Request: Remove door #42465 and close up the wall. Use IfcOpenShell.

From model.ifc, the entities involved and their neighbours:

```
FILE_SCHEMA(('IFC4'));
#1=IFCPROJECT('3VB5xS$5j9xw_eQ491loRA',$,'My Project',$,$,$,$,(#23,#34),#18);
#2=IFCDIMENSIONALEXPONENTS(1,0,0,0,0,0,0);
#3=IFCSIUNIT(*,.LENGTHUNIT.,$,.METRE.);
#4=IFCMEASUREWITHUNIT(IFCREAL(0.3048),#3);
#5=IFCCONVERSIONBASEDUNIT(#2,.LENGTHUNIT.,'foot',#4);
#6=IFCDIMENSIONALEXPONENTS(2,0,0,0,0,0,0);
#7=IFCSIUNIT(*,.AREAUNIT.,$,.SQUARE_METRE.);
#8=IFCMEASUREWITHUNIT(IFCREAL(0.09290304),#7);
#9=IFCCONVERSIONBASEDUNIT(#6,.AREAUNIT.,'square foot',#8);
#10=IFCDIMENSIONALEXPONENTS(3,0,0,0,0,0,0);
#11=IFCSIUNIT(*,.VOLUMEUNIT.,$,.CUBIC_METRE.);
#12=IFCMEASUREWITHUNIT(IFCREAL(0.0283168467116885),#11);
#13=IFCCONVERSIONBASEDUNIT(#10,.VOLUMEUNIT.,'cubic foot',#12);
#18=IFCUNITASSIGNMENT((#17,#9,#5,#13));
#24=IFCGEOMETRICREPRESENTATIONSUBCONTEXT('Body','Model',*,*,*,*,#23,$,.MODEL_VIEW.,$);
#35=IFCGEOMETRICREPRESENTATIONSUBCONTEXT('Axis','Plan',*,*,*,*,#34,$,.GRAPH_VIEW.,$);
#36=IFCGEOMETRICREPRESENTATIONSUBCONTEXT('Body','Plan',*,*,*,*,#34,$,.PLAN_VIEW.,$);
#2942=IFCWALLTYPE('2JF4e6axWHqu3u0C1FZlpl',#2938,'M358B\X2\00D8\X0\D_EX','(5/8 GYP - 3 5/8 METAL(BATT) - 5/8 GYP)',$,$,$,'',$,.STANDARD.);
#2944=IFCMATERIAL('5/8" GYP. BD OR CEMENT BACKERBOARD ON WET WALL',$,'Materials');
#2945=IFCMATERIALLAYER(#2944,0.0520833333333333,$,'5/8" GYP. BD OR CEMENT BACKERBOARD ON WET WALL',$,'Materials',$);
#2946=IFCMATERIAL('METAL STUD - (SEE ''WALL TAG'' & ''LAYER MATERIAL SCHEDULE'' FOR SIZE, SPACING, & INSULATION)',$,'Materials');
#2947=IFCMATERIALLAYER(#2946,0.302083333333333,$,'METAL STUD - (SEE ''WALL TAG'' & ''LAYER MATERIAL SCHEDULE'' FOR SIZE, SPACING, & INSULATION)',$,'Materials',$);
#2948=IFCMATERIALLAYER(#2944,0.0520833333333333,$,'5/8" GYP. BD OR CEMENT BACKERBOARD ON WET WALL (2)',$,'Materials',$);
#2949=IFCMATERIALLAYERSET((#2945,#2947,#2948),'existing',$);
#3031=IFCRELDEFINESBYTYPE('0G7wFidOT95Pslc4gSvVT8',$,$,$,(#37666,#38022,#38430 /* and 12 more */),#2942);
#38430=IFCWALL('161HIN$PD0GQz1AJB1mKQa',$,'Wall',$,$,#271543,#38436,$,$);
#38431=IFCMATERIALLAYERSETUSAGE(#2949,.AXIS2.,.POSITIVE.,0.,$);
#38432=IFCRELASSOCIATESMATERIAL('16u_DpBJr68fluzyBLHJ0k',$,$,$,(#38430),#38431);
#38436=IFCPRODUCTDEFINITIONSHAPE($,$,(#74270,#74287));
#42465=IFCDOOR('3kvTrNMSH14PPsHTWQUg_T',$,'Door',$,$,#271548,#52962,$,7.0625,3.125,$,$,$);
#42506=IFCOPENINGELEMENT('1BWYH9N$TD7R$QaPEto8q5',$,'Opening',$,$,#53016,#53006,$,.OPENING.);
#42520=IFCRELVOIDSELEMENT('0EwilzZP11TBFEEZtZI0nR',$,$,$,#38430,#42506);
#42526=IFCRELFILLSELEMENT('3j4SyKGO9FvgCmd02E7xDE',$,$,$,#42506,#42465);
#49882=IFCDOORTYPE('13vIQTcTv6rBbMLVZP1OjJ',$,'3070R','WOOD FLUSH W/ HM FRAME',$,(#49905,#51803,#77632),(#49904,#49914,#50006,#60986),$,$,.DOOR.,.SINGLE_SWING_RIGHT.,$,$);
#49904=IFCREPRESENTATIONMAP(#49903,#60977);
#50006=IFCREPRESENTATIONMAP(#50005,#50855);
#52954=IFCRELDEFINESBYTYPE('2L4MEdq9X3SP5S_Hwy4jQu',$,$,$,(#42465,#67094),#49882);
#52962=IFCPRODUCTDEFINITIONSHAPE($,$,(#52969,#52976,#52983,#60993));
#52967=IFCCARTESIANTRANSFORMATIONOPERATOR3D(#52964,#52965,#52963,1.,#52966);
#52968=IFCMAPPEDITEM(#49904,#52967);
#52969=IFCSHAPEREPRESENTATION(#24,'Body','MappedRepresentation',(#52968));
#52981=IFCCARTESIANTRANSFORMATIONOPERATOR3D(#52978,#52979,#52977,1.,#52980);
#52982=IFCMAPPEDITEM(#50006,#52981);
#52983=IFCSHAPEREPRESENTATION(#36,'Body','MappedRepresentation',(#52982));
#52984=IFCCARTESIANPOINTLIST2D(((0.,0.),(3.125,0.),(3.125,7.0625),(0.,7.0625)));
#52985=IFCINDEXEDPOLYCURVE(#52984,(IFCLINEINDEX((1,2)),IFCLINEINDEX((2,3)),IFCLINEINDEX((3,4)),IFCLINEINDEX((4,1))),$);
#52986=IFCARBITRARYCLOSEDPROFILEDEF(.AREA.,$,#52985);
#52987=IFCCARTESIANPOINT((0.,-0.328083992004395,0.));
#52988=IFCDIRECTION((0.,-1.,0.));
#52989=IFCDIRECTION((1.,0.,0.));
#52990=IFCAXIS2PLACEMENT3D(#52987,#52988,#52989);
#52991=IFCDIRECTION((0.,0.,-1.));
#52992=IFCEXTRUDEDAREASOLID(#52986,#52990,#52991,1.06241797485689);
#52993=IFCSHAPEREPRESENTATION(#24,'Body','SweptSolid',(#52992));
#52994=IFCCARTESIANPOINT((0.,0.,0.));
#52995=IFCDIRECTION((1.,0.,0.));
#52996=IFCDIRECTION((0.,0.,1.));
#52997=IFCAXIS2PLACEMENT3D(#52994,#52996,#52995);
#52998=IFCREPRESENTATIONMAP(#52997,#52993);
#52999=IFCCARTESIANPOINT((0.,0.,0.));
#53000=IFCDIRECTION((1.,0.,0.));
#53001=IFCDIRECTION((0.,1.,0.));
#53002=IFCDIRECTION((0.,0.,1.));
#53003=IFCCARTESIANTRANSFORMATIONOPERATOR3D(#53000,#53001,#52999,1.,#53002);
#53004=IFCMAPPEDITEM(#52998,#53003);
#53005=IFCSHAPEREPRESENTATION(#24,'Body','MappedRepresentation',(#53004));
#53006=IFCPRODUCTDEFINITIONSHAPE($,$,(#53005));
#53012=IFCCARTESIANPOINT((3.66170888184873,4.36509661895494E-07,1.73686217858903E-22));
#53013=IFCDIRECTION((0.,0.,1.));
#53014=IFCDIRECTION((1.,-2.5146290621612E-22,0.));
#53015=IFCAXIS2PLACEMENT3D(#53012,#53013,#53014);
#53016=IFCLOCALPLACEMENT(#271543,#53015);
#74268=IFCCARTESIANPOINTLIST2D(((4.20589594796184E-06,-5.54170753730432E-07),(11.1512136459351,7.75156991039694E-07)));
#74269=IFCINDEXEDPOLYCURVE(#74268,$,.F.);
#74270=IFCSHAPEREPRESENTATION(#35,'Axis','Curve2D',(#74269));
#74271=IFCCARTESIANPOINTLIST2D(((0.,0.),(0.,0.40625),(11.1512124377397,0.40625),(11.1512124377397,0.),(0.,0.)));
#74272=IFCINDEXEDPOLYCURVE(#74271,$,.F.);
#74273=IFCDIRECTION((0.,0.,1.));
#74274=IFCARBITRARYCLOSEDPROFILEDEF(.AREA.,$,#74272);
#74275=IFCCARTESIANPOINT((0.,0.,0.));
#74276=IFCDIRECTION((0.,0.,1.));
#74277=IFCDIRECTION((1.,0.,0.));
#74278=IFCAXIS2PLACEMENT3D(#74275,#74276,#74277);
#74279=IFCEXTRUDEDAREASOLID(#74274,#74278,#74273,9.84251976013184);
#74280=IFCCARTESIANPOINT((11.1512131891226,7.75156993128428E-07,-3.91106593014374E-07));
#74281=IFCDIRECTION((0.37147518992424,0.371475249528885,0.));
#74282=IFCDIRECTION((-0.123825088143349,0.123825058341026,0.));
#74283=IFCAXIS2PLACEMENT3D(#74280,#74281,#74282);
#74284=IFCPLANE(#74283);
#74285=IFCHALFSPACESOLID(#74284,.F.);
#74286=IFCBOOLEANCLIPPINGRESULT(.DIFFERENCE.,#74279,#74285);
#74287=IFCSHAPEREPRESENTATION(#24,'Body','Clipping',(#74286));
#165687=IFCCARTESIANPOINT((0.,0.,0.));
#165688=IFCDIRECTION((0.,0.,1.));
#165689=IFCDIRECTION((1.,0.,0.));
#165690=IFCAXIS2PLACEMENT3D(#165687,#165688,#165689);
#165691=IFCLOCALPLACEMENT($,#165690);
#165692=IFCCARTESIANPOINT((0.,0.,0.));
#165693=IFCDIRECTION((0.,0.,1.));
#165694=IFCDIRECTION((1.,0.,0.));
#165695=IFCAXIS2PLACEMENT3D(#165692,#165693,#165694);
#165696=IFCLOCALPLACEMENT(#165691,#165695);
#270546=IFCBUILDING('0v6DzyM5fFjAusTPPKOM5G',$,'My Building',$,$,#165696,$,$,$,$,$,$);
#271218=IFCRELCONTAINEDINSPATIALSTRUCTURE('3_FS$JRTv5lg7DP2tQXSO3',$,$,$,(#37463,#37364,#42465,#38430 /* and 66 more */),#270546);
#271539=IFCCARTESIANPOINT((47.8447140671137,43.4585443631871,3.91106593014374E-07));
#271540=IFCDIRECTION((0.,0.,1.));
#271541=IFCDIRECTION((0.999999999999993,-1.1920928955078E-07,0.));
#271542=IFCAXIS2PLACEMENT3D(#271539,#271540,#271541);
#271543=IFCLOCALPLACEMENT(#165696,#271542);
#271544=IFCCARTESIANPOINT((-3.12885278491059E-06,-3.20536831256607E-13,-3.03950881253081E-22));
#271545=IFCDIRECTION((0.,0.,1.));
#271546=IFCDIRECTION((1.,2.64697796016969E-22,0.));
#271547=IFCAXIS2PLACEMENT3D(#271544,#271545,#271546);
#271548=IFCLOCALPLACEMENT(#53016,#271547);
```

```python
import ifcopenshell
import ifcopenshell.api.feature
import ifcopenshell.api.root
import ifcopenshell.geom
import ifcopenshell.util.shape

model = ifcopenshell.open("model.ifc")
settings = ifcopenshell.geom.settings()


def volume(element):
    """Net volume in cubic metres, openings subtracted."""
    shape = ifcopenshell.geom.create_shape(settings, element)
    return ifcopenshell.util.shape.get_volume(shape.geometry)


door = model.by_guid("3kvTrNMSH14PPsHTWQUg_T")
opening = door.FillsVoids[0].RelatingOpeningElement
wall = opening.VoidsElements[0].RelatingBuildingElement
before = volume(wall)

ifcopenshell.api.root.remove_product(model, product=door)
ifcopenshell.api.feature.remove_feature(model, feature=opening)

after = volume(wall)

print(f"wall volume {before:.3f} -> {after:.3f} m3")

model.write("model_updated.ifc")
```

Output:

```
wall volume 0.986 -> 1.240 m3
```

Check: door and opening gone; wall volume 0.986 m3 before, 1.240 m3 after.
